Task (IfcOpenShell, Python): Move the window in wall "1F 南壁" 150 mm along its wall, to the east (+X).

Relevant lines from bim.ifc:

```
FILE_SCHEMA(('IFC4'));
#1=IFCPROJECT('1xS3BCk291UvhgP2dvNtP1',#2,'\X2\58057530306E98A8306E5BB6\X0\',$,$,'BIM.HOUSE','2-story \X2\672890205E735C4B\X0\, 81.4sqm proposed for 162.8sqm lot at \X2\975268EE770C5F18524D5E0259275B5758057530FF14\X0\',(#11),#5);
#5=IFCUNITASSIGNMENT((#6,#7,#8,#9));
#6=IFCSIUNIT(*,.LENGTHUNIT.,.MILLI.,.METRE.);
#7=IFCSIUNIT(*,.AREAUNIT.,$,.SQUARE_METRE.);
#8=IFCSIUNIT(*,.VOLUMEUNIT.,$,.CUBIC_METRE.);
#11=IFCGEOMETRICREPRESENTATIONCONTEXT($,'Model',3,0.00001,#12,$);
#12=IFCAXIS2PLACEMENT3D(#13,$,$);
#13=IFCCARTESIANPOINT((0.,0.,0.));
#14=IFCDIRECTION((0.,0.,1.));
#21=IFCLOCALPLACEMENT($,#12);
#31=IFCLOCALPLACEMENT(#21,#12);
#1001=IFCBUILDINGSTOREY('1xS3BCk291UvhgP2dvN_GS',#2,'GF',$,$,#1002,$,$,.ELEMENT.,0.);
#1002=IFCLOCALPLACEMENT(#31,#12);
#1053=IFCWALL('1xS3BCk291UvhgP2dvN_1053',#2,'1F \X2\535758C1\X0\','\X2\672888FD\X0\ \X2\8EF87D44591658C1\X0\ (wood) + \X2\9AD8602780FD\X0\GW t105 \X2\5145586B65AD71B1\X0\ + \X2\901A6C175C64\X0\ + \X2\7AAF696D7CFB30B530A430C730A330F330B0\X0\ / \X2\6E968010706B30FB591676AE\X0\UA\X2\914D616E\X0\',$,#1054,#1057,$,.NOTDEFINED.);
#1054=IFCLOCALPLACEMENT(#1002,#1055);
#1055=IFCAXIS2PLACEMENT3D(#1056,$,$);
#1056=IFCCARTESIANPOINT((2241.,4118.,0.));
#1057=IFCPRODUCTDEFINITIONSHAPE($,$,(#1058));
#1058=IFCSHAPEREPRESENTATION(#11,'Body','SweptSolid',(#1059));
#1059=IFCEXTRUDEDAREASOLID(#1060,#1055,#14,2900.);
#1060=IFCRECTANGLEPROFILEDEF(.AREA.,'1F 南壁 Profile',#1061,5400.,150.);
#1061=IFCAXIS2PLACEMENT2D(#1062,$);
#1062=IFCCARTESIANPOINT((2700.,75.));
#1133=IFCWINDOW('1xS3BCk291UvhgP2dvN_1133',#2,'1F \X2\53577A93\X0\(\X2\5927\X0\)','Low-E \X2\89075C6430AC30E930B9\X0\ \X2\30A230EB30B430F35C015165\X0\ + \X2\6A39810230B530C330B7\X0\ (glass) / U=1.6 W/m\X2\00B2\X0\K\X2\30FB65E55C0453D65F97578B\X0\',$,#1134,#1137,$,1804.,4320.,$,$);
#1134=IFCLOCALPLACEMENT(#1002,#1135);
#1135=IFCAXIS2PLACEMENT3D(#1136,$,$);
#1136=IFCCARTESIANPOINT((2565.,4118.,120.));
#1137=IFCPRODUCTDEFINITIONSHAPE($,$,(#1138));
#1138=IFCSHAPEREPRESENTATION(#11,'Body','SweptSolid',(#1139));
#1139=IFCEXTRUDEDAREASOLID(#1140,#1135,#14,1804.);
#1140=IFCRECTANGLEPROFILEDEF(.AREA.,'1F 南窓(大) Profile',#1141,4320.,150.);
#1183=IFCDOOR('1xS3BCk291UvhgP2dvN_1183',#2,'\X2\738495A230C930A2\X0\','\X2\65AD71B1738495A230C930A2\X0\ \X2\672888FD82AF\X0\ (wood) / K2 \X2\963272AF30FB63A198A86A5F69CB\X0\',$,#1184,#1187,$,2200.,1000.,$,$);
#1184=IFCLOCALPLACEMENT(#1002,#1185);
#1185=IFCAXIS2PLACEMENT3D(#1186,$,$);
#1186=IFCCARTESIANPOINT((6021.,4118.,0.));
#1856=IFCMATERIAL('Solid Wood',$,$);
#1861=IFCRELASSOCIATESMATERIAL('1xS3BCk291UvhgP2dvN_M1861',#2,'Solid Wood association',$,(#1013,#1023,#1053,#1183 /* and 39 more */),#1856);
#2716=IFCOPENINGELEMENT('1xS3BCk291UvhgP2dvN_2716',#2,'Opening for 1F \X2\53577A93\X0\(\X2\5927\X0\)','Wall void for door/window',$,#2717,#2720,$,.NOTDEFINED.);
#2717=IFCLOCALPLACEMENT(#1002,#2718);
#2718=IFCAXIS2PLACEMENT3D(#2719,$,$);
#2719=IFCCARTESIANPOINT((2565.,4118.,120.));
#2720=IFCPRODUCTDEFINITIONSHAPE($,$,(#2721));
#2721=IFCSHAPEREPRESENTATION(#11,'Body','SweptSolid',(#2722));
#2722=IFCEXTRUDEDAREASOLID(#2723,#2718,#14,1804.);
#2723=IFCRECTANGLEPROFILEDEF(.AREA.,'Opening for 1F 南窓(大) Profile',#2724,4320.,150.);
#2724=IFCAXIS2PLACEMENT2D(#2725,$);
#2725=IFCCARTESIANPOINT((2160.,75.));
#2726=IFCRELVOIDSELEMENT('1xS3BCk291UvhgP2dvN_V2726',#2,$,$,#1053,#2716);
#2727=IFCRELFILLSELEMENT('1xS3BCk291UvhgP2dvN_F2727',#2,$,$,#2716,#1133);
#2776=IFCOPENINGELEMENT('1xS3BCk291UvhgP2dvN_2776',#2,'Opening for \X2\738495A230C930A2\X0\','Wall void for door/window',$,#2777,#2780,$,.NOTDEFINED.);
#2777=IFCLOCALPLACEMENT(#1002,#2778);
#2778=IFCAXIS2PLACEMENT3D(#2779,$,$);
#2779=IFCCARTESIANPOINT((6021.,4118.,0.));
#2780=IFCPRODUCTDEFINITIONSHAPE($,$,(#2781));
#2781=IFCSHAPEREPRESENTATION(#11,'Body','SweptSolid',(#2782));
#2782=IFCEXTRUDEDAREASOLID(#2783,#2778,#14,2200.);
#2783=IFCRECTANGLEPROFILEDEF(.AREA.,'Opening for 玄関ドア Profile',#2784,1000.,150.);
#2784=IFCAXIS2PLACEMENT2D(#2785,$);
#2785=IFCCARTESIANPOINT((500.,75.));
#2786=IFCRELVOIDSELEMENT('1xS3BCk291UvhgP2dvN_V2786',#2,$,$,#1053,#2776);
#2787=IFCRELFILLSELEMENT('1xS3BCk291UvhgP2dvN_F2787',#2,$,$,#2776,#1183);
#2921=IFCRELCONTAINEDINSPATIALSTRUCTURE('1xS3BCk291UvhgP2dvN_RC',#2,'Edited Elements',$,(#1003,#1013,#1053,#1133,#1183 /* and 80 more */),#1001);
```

```python
import ifcopenshell
import ifcopenshell.api.geometry
import ifcopenshell.util.placement

model = ifcopenshell.open("bim.ifc")

window = model.by_guid("1xS3BCk291UvhgP2dvN_1133")
opening = window.FillsVoids[0].RelatingOpeningElement
wall = opening.VoidsElements[0].RelatingBuildingElement

wall_matrix = ifcopenshell.util.placement.get_local_placement(wall.ObjectPlacement)
shift = wall_matrix[:3, 0] * 150.0
before = ifcopenshell.util.placement.get_local_placement(window.ObjectPlacement)[:3, 3].copy()

# The window is not placed relative to its opening, so move both.
for product in (opening, window):
    matrix = ifcopenshell.util.placement.get_local_placement(product.ObjectPlacement)
    matrix[:3, 3] += shift
    ifcopenshell.api.geometry.edit_object_placement(model, product=product, matrix=matrix, is_si=False)

after = ifcopenshell.util.placement.get_local_placement(window.ObjectPlacement)[:3, 3]
print("window moved by", (after - before).round(3) + 0.0)

model.write("bim-out.ifc")
```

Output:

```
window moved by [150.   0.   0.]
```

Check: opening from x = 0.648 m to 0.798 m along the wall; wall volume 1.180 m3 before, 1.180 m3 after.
